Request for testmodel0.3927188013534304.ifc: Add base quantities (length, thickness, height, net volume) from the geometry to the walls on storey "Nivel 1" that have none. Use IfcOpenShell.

First a look at what the model holds.

```python
import ifcopenshell
import ifcopenshell.util.element
import ifcopenshell.util.unit

model = ifcopenshell.open("testmodel0.3927188013534304.ifc")
print(model.schema)
for unit_type in ("LENGTHUNIT", "AREAUNIT", "VOLUMEUNIT"):
    print(unit_type, ifcopenshell.util.unit.calculate_unit_scale(model, unit_type))
storey = next(s for s in model.by_type("IfcBuildingStorey") if s.Name == "Nivel 1")
walls = [e for e in ifcopenshell.util.element.get_decomposition(storey) if e.is_a("IfcWall")]
for e in sorted(walls, key=lambda e: e.id()):
    print(e.id(), e.is_a(), e.Name, list(ifcopenshell.util.element.get_psets(e, qtos_only=True)), sep=" | ")
```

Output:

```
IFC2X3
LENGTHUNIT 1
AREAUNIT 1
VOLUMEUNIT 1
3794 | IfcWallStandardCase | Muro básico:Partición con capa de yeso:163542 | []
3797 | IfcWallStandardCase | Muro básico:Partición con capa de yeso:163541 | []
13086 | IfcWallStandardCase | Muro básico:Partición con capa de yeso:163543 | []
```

```python
import ifcopenshell
import ifcopenshell.api.pset
import ifcopenshell.geom
import ifcopenshell.util.element
import ifcopenshell.util.shape
import ifcopenshell.util.unit

model = ifcopenshell.open("testmodel0.3927188013534304.ifc")
unit_scale = ifcopenshell.util.unit.calculate_unit_scale(model)
volume_scale = ifcopenshell.util.unit.calculate_unit_scale(model, "VOLUMEUNIT")
settings = ifcopenshell.geom.settings()

storey = next(s for s in model.by_type("IfcBuildingStorey") if s.Name == "Nivel 1")
walls = [e for e in ifcopenshell.util.element.get_decomposition(storey) if e.is_a("IfcWall")]

for e in sorted(walls, key=lambda e: e.id()):
    if ifcopenshell.util.element.get_psets(e, qtos_only=True, should_inherit=False):
        continue
    # Geometry comes back in metres, in the element's own axes.
    shape = ifcopenshell.geom.create_shape(settings, e)
    values = {
        "Length": ifcopenshell.util.shape.get_x(shape.geometry) / unit_scale,
        "Width": ifcopenshell.util.shape.get_y(shape.geometry) / unit_scale,
        "Height": ifcopenshell.util.shape.get_z(shape.geometry) / unit_scale,
        "NetVolume": ifcopenshell.util.shape.get_volume(shape.geometry) / volume_scale,
    }
    qto = ifcopenshell.api.pset.add_qto(model, product=e, name="BaseQuantities")
    ifcopenshell.api.pset.edit_qto(model, qto=qto, properties=values)
    print(e.id(), {k: round(v, 3) for k, v in values.items()})

model.write("testmodel0.3927188013534304-out.ifc")
```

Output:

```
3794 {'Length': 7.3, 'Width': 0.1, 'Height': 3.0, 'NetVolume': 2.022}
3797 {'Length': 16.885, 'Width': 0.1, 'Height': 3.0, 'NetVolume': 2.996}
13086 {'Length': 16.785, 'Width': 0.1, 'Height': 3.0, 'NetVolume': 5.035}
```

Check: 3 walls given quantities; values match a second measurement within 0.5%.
